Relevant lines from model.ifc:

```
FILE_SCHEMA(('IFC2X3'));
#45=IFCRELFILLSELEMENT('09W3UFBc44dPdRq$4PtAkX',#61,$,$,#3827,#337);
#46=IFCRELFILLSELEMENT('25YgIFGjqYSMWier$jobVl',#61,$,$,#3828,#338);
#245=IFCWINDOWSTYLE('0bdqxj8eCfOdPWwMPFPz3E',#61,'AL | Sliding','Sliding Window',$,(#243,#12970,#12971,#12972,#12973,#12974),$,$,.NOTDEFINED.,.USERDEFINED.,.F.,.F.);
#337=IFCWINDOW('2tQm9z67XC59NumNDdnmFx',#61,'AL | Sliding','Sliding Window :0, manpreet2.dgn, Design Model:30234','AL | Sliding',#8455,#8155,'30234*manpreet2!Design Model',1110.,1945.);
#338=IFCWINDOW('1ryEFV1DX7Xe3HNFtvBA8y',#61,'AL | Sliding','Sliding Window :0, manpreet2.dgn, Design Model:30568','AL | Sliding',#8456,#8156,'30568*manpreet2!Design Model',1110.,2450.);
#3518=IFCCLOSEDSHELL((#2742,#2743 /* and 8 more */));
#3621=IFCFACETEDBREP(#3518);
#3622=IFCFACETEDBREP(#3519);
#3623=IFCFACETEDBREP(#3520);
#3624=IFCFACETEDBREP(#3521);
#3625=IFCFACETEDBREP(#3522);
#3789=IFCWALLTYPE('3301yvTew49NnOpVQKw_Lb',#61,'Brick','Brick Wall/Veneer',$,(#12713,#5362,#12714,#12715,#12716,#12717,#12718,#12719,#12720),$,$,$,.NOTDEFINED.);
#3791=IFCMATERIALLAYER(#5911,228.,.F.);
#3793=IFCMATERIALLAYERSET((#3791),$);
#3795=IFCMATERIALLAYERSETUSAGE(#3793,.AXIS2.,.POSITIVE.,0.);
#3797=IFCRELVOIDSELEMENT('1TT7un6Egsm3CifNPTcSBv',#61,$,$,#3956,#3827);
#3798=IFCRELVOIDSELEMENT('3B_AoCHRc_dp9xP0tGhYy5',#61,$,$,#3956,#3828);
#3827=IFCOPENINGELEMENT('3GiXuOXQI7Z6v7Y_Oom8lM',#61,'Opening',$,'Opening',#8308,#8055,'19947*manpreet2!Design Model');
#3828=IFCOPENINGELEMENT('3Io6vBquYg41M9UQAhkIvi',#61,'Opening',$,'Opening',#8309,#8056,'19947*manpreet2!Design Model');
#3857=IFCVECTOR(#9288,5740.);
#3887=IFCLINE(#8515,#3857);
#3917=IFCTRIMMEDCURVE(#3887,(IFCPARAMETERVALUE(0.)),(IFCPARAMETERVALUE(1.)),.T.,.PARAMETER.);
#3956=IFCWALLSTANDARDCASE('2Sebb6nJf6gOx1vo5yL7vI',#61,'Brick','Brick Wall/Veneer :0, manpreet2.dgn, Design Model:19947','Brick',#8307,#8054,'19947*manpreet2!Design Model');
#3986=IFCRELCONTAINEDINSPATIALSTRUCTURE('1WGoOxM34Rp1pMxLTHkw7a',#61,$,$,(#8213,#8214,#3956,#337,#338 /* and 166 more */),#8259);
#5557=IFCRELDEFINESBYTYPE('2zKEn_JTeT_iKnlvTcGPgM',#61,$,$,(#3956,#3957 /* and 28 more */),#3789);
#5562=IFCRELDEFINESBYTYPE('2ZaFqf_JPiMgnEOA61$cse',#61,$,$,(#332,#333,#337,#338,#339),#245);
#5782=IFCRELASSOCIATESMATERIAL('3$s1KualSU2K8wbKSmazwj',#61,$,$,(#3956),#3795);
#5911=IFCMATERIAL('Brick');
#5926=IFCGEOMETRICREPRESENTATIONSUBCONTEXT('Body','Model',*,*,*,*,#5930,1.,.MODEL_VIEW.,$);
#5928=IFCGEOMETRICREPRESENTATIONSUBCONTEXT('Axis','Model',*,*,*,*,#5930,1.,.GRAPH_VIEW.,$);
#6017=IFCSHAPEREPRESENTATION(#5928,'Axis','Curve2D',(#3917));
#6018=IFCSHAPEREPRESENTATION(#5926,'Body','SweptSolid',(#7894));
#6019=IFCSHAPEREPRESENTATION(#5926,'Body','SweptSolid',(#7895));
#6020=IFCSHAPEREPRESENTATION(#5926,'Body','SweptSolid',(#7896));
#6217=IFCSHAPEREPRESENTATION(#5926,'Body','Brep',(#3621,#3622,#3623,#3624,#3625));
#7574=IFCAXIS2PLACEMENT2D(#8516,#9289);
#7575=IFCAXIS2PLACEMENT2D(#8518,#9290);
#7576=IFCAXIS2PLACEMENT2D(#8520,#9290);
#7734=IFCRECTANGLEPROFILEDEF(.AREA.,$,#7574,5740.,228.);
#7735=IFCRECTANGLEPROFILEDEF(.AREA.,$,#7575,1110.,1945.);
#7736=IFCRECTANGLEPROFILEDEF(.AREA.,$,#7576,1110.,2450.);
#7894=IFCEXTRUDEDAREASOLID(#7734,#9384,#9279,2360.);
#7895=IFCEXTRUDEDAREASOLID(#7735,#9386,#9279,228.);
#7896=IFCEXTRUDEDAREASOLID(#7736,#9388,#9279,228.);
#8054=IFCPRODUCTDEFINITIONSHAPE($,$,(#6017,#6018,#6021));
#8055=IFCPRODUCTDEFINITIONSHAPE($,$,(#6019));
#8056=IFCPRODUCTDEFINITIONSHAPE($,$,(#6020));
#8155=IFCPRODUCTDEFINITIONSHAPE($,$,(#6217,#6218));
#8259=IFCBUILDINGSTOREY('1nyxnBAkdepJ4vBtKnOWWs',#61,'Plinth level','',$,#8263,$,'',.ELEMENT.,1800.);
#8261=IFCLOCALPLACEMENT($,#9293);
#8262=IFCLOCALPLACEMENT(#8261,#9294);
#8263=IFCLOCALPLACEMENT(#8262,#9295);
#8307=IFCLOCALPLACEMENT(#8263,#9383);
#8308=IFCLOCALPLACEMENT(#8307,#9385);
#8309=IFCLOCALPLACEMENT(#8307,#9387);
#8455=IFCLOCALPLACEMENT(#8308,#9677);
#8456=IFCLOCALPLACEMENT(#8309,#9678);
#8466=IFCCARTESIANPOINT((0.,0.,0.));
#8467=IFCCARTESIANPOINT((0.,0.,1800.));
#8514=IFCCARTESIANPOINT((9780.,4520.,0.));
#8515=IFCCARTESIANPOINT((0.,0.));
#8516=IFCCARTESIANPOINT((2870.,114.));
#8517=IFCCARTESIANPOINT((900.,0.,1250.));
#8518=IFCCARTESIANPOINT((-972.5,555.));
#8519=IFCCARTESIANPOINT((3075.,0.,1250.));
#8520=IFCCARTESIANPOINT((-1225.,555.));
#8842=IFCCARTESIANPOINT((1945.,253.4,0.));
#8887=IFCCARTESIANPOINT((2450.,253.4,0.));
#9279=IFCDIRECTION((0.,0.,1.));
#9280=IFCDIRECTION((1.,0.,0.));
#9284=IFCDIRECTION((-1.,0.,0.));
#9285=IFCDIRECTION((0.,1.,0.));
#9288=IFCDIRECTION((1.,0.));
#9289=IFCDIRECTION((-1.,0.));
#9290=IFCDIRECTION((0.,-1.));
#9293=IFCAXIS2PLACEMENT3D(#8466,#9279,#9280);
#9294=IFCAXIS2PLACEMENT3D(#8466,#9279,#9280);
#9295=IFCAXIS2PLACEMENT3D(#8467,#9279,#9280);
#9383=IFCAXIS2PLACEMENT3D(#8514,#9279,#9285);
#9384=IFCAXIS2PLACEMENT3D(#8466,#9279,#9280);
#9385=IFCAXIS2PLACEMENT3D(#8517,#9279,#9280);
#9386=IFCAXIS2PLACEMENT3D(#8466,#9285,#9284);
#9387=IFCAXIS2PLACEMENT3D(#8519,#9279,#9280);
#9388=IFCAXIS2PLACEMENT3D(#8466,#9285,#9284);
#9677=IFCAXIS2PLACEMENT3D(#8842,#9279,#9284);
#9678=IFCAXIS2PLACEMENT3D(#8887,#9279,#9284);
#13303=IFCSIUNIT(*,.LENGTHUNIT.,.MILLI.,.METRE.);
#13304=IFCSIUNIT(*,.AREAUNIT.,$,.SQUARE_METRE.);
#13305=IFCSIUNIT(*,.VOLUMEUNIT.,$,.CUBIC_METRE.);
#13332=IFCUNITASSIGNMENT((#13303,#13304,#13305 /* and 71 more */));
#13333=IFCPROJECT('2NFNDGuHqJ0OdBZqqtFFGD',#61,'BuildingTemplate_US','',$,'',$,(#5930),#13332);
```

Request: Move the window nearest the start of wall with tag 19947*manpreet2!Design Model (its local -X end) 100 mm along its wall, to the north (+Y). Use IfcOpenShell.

```python
import ifcopenshell
import ifcopenshell.api.geometry
import ifcopenshell.util.placement

model = ifcopenshell.open("model.ifc")

window = model.by_guid("2tQm9z67XC59NumNDdnmFx")
opening = window.FillsVoids[0].RelatingOpeningElement
wall = opening.VoidsElements[0].RelatingBuildingElement

wall_matrix = ifcopenshell.util.placement.get_local_placement(wall.ObjectPlacement)
shift = wall_matrix[:3, 0] * 100.0
before = ifcopenshell.util.placement.get_local_placement(window.ObjectPlacement)[:3, 3].copy()

# The window is placed relative to its opening, so it follows when the opening moves.
matrix = ifcopenshell.util.placement.get_local_placement(opening.ObjectPlacement)
matrix[:3, 3] += shift
ifcopenshell.api.geometry.edit_object_placement(
    model, product=opening, matrix=matrix, is_si=False, should_transform_children=True
)

after = ifcopenshell.util.placement.get_local_placement(window.ObjectPlacement)[:3, 3]
print("window moved by", (after - before).round(3) + 0.0)

model.write("model_edited.ifc")
```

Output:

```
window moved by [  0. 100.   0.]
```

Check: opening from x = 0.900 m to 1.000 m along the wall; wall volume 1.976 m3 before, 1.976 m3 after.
